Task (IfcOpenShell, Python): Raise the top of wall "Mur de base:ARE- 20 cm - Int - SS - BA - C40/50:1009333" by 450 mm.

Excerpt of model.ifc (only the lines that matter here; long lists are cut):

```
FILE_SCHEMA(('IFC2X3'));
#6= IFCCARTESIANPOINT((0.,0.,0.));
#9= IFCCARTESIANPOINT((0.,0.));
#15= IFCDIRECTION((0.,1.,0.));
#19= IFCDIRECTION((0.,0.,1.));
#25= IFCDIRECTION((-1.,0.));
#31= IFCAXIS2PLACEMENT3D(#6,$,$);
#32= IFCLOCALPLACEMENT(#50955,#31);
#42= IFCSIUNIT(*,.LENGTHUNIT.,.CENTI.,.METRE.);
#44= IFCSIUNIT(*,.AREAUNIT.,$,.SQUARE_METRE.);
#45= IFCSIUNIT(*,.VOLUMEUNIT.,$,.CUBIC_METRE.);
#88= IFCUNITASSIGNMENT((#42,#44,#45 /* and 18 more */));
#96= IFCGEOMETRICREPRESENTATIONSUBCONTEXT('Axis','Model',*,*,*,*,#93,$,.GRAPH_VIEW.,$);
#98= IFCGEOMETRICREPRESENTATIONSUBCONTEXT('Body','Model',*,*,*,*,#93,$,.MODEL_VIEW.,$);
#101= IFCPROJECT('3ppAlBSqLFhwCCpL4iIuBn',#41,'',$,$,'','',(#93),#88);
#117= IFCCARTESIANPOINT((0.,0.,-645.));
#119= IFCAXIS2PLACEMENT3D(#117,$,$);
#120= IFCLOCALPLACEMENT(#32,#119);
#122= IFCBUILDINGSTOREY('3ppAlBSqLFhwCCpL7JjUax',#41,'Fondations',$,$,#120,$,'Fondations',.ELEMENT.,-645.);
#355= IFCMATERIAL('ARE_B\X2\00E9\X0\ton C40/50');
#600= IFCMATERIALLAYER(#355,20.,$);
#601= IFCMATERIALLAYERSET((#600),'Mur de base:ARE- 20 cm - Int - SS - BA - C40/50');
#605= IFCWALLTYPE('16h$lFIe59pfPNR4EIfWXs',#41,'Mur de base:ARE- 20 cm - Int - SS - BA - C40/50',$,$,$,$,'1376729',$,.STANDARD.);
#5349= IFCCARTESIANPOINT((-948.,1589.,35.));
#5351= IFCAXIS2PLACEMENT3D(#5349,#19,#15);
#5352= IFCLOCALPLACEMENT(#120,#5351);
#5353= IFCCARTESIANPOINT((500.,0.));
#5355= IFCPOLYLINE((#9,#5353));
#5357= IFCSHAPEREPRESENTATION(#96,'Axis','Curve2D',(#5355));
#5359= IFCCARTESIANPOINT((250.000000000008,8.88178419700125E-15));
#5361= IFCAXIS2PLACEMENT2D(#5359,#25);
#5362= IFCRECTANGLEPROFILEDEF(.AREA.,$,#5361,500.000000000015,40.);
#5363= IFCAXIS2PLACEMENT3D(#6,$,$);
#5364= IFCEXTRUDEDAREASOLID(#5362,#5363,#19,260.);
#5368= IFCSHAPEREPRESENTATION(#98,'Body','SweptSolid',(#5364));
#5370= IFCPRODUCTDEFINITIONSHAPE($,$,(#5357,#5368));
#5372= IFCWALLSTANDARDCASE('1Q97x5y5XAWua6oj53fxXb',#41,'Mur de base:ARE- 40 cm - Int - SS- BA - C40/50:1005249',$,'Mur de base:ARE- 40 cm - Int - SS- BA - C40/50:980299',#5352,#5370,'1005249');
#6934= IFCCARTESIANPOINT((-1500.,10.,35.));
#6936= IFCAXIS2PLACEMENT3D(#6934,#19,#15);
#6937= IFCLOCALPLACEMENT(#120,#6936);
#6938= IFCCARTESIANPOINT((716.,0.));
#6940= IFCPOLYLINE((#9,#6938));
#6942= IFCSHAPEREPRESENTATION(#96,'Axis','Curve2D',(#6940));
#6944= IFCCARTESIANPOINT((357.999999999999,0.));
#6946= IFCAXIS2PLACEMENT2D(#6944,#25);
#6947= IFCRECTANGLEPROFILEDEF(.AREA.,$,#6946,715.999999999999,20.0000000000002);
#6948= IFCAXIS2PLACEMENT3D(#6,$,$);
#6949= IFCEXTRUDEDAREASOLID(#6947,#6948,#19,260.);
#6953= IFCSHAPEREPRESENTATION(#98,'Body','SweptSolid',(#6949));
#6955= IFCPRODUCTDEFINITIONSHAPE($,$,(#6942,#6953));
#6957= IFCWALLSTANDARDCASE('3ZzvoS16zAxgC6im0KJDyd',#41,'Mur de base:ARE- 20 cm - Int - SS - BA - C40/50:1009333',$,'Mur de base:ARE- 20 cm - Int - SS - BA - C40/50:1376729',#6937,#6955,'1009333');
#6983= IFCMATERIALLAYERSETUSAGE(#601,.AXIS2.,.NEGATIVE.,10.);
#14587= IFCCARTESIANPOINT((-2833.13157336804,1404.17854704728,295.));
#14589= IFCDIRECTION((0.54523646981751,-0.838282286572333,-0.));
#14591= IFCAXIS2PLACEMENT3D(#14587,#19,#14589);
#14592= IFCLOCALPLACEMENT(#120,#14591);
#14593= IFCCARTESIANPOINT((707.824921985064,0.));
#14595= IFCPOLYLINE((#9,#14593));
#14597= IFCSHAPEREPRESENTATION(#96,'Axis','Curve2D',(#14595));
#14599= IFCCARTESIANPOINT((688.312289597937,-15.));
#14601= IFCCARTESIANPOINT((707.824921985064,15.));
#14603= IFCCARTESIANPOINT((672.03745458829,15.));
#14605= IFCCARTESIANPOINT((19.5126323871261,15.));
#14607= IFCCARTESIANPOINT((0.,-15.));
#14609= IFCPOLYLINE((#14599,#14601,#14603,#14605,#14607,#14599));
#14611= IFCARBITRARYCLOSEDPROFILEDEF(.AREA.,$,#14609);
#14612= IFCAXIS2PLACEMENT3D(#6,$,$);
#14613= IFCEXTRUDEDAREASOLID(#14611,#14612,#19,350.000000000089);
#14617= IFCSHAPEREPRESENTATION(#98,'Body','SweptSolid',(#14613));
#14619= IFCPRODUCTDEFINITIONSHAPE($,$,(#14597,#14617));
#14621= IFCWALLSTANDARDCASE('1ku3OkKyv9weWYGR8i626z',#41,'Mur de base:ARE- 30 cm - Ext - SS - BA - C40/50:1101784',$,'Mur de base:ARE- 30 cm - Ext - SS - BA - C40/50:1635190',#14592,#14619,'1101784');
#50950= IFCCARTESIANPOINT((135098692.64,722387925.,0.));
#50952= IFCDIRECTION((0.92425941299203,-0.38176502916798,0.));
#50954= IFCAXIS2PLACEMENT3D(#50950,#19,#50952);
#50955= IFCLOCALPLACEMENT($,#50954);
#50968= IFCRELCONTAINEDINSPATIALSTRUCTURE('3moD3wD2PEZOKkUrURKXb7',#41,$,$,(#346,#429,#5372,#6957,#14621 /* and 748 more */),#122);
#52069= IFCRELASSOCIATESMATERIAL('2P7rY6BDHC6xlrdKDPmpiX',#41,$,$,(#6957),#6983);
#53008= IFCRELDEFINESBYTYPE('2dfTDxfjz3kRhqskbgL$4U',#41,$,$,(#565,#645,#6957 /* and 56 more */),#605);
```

```python
import ifcopenshell
import ifcopenshell.geom
import ifcopenshell.util.representation
import ifcopenshell.util.shape
import ifcopenshell.util.unit

model = ifcopenshell.open("model.ifc")
unit_scale = ifcopenshell.util.unit.calculate_unit_scale(model)
settings = ifcopenshell.geom.settings()


def volume(element):
    """Net volume in cubic metres, openings subtracted."""
    shape = ifcopenshell.geom.create_shape(settings, element)
    return ifcopenshell.util.shape.get_volume(shape.geometry)


wall = model.by_id(6957)
before = volume(wall)

body = ifcopenshell.util.representation.get_representation(wall, "Model", "Body")
solid = body.Items[0]
old_height = solid.Depth
solid.Depth += 0.45 / unit_scale
after = volume(wall)

print(f"height {old_height:g} -> {solid.Depth:g}, volume {before:.3f} -> {after:.3f} m3")

model.write("model_rev.ifc")
```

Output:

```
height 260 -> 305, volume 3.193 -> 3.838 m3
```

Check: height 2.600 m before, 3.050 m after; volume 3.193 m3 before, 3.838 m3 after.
